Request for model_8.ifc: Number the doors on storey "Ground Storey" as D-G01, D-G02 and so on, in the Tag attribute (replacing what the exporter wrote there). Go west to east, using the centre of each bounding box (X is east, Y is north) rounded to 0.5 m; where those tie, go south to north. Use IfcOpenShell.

First a look at what the model holds.

```python
import ifcopenshell
import ifcopenshell.util.element
import ifcopenshell.util.placement

model = ifcopenshell.open("model_8.ifc")
print(model.schema)
storey = next(s for s in model.by_type("IfcBuildingStorey") if s.Name == "Ground Storey")
doors = [e for e in ifcopenshell.util.element.get_decomposition(storey) if e.is_a("IfcDoor")]
for e in sorted(doors, key=lambda e: e.id()):
    origin = ifcopenshell.util.placement.get_local_placement(e.ObjectPlacement)[:3, 3]
    print(e.id(), e.Tag, e.Name, origin.round(2) + 0.0, sep=" | ")
```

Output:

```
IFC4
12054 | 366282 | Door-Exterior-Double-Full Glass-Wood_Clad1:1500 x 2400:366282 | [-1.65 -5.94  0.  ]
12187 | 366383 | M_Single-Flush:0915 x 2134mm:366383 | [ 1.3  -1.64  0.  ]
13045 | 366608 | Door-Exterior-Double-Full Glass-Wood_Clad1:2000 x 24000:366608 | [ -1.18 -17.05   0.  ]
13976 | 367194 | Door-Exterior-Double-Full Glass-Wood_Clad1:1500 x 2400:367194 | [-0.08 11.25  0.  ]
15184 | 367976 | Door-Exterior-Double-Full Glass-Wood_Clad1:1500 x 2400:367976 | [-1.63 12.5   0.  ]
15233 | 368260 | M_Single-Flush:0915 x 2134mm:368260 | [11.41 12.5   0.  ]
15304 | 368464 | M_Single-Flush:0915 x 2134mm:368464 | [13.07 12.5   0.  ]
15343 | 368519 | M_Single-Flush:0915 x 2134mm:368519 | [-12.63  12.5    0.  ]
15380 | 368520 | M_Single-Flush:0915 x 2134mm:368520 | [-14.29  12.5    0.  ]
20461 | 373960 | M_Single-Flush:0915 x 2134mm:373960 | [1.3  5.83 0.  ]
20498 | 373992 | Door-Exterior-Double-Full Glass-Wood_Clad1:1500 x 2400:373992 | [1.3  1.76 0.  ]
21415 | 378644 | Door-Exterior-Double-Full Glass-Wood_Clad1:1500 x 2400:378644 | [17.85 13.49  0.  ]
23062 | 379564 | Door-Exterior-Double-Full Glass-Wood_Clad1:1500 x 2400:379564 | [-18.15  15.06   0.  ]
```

```python
import ifcopenshell
import ifcopenshell.geom
import ifcopenshell.util.element
import ifcopenshell.util.shape

model = ifcopenshell.open("model_8.ifc")
settings = ifcopenshell.geom.settings()
settings.set("use-world-coords", True)


def centre(element):
    shape = ifcopenshell.geom.create_shape(settings, element)
    return ifcopenshell.util.shape.get_bbox_centroid(shape.geometry)


storey = next(s for s in model.by_type("IfcBuildingStorey") if s.Name == "Ground Storey")
doors = [e for e in ifcopenshell.util.element.get_decomposition(storey) if e.is_a("IfcDoor")]

# Insertion points can sit at a corner or the storey origin, so sort by the geometry (in metres).
centres = {e: centre(e) for e in doors}
doors.sort(key=lambda e: (round(centres[e][0] / 0.5), centres[e][1]))

for i, e in enumerate(doors, start=1):
    number = f"D-G{i:02d}"
    e.Tag = number
    print(e.id(), number)

model.write("model_8_v2.ifc")
```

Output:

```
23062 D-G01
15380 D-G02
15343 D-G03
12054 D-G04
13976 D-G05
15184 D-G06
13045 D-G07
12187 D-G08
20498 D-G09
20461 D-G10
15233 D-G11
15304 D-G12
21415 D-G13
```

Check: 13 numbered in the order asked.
